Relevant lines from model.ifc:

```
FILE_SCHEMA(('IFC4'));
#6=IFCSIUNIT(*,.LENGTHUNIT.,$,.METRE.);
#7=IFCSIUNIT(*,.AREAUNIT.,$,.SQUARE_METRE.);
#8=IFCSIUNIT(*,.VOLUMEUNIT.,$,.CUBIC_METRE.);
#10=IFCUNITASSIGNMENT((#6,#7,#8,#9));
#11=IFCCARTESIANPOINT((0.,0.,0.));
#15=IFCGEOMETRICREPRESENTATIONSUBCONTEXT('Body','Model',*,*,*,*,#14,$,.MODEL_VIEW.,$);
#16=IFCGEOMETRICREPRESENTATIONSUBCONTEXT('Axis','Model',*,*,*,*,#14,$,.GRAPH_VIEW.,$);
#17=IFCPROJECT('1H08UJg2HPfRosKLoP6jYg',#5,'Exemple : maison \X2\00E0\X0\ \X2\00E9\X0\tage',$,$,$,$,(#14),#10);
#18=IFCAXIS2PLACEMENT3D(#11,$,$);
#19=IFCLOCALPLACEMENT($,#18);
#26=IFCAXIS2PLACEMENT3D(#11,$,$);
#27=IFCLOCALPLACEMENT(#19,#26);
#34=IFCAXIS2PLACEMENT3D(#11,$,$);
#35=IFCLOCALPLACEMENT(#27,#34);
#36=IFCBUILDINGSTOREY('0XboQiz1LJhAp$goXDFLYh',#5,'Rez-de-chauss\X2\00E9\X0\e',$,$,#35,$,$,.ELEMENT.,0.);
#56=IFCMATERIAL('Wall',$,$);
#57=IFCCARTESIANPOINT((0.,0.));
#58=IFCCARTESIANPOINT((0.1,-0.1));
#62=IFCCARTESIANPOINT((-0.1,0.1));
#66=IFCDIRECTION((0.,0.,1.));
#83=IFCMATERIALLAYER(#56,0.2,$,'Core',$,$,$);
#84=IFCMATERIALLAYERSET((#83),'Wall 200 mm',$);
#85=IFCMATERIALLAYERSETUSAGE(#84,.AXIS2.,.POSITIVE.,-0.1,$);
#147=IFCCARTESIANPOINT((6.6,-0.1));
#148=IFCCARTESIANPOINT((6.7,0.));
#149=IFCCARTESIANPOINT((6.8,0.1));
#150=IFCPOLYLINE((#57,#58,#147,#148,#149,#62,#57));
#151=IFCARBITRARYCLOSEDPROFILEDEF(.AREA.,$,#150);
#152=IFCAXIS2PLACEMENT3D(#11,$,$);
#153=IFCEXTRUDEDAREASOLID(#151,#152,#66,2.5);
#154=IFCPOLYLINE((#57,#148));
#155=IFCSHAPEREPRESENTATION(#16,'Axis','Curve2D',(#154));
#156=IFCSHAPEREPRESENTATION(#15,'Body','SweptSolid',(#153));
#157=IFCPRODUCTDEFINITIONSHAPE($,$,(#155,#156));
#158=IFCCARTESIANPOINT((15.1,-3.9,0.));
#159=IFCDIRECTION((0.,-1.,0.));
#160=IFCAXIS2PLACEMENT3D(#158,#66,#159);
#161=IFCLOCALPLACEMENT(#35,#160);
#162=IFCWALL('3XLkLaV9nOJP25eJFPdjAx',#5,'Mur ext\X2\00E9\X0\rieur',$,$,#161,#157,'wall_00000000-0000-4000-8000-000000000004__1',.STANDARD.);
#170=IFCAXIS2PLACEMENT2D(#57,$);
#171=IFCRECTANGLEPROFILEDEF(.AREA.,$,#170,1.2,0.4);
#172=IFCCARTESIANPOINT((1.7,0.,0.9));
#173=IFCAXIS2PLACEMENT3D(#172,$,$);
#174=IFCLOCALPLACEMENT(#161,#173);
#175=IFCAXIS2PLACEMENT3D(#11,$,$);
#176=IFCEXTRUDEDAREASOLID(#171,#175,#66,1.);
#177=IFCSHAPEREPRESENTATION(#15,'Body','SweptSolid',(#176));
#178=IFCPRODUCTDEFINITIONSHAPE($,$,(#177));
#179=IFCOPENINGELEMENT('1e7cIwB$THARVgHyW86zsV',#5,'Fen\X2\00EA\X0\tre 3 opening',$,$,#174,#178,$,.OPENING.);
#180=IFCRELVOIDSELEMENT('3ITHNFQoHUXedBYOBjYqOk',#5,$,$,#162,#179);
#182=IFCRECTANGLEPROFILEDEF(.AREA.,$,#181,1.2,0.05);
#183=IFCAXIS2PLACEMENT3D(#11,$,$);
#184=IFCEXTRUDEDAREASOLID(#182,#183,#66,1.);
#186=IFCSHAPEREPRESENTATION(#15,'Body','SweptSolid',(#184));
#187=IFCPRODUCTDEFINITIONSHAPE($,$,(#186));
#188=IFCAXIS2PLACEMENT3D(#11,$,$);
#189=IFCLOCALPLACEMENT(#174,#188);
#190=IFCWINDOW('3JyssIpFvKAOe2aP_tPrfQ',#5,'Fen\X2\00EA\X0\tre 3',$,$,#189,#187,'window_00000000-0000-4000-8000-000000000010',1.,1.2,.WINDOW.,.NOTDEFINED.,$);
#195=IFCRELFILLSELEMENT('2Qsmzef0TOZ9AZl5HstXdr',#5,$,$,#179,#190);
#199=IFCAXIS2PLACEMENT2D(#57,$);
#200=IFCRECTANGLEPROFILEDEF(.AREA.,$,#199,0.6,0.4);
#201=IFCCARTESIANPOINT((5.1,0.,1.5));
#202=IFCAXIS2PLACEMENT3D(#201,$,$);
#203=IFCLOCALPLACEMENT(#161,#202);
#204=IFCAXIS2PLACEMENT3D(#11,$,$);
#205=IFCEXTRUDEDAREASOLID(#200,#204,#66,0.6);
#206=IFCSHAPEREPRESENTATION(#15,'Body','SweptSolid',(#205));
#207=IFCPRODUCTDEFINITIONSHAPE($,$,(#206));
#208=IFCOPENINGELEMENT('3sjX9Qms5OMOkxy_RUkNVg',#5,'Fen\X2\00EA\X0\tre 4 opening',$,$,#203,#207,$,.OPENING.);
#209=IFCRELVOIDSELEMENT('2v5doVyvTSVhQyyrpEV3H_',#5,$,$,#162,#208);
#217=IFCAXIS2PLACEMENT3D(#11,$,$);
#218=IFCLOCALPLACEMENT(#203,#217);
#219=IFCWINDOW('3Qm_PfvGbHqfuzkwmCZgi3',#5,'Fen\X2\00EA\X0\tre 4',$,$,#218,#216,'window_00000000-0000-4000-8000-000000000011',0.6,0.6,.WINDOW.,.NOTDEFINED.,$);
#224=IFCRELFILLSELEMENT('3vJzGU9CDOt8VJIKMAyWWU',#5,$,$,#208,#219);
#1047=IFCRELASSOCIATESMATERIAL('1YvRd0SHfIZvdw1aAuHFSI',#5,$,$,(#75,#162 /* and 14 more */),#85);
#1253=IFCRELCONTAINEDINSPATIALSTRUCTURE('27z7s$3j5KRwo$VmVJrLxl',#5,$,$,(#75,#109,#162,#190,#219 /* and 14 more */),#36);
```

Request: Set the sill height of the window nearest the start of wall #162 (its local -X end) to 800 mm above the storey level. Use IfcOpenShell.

```python
import numpy as np
import ifcopenshell
import ifcopenshell.api.geometry
import ifcopenshell.geom
import ifcopenshell.util.element
import ifcopenshell.util.placement
import ifcopenshell.util.shape
import ifcopenshell.util.unit

model = ifcopenshell.open("model.ifc")
unit_scale = ifcopenshell.util.unit.calculate_unit_scale(model)

window = model.by_guid("3JyssIpFvKAOe2aP_tPrfQ")
opening = window.FillsVoids[0].RelatingOpeningElement
storey = ifcopenshell.util.element.get_container(window, ifc_class="IfcBuildingStorey")
level = ifcopenshell.util.placement.get_local_placement(storey.ObjectPlacement)[2, 3]

# The opening's origin need not be at the sill, so measure its lowest point.
shape = ifcopenshell.geom.create_shape(ifcopenshell.geom.settings(), opening)
bottom = ifcopenshell.util.shape.get_shape_bottom_elevation(shape, shape.geometry) / unit_scale
dz = level + 0.8 / unit_scale - bottom

shift = np.array([0.0, 0.0, dz])
# The window is placed relative to its opening, so it follows when the opening moves.
matrix = ifcopenshell.util.placement.get_local_placement(opening.ObjectPlacement)
matrix[:3, 3] += shift
ifcopenshell.api.geometry.edit_object_placement(
    model, product=opening, matrix=matrix, is_si=False, should_transform_children=True
)

print(f"moved by {dz * unit_scale:+.3f} m")

model.write("model_edited.ifc")
```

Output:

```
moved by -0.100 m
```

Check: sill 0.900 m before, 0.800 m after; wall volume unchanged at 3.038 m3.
